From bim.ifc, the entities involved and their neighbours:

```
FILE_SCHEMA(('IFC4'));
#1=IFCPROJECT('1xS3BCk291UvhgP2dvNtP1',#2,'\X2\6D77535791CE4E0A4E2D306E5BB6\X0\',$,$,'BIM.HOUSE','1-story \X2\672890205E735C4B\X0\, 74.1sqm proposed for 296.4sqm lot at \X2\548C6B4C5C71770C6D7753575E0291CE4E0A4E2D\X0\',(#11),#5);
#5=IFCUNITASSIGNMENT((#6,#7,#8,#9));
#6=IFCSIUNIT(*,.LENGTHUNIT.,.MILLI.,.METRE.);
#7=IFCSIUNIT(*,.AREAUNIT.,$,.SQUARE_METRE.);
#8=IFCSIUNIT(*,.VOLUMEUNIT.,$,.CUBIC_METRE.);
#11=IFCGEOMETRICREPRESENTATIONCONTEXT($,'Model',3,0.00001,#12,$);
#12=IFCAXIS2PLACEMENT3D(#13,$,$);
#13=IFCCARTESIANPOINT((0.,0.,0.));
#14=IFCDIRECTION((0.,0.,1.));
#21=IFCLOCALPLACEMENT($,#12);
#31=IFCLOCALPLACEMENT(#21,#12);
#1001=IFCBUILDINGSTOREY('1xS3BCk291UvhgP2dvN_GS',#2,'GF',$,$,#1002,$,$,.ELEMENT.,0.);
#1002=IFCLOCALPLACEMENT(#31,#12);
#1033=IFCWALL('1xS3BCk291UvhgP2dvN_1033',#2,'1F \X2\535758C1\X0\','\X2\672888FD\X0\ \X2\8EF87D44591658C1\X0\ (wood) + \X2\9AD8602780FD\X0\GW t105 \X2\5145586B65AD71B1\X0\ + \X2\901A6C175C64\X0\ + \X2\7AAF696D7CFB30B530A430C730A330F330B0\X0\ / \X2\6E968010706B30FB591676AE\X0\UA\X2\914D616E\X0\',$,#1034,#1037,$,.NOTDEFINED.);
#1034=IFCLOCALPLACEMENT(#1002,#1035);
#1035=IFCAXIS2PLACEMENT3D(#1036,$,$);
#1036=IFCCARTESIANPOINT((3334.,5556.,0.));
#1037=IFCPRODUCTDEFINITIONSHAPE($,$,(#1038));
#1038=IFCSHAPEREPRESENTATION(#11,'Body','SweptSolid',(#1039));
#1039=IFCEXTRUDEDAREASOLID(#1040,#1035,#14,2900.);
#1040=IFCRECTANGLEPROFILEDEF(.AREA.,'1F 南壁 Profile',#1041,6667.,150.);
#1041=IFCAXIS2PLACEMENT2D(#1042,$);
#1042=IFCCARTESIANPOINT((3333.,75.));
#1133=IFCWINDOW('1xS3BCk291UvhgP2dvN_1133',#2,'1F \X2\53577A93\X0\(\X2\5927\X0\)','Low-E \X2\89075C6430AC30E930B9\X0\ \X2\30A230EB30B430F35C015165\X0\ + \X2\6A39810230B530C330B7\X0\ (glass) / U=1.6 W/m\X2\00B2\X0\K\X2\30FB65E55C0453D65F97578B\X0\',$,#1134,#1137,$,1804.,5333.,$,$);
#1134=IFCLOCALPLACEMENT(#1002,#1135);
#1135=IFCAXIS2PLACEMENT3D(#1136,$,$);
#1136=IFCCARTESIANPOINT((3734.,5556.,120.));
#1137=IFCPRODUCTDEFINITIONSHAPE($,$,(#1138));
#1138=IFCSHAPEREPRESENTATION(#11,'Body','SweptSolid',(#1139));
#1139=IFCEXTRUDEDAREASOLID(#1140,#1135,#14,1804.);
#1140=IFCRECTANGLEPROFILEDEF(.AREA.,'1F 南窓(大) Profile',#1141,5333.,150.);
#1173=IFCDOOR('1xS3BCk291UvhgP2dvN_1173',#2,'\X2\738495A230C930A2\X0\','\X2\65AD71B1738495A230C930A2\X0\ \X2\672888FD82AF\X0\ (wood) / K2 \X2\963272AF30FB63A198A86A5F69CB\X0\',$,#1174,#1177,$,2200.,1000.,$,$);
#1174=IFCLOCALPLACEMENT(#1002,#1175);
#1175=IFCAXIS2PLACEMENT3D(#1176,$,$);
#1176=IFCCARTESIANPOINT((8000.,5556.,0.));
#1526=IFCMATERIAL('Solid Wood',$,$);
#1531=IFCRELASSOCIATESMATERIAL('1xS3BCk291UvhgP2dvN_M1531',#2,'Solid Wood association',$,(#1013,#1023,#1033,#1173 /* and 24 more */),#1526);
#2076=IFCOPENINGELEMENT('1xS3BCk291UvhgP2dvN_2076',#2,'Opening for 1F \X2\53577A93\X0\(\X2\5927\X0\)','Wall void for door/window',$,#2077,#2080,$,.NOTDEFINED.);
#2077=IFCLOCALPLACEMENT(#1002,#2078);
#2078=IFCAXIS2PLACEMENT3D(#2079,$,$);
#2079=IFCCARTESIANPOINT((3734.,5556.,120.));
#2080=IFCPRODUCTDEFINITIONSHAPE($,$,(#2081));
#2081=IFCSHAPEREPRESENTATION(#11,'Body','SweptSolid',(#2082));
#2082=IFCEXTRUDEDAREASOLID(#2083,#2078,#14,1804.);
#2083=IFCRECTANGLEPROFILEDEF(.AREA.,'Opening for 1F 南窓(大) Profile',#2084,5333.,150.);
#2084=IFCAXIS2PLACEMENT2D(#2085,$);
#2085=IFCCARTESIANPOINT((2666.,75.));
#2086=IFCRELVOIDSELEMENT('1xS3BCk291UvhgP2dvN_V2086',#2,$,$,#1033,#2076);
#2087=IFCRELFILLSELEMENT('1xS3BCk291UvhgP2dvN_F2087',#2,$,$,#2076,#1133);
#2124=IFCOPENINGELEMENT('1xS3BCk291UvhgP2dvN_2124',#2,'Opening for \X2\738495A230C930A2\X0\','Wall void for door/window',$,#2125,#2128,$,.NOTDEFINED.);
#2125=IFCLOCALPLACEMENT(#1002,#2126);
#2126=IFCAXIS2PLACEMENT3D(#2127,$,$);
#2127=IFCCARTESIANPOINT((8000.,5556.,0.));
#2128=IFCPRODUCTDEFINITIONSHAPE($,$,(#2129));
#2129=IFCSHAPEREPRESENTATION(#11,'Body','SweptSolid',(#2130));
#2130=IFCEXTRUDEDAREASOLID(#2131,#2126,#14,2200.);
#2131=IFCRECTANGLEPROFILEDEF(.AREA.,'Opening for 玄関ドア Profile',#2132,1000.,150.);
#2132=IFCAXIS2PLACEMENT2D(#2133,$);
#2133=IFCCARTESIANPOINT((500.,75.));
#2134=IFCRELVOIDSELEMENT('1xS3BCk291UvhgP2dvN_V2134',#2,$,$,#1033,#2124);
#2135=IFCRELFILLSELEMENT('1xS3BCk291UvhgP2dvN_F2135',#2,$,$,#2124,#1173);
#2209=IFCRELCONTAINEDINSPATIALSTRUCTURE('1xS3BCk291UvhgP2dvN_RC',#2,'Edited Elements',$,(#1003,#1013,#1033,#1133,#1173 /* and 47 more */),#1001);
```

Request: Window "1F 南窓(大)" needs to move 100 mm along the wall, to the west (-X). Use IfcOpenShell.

```python
import ifcopenshell
import ifcopenshell.api.geometry
import ifcopenshell.util.placement

model = ifcopenshell.open("bim.ifc")

window = model.by_id(1133)
opening = window.FillsVoids[0].RelatingOpeningElement
wall = opening.VoidsElements[0].RelatingBuildingElement

wall_matrix = ifcopenshell.util.placement.get_local_placement(wall.ObjectPlacement)
shift = wall_matrix[:3, 0] * -100.0
before = ifcopenshell.util.placement.get_local_placement(window.ObjectPlacement)[:3, 3].copy()

# The window is not placed relative to its opening, so move both.
for product in (opening, window):
    matrix = ifcopenshell.util.placement.get_local_placement(product.ObjectPlacement)
    matrix[:3, 3] += shift
    ifcopenshell.api.geometry.edit_object_placement(model, product=product, matrix=matrix, is_si=False)

after = ifcopenshell.util.placement.get_local_placement(window.ObjectPlacement)[:3, 3]
print("window moved by", (after - before).round(3) + 0.0)

model.write("bim_v2.ifc")
```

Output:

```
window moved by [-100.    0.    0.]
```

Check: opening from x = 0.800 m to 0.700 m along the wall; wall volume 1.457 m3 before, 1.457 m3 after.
